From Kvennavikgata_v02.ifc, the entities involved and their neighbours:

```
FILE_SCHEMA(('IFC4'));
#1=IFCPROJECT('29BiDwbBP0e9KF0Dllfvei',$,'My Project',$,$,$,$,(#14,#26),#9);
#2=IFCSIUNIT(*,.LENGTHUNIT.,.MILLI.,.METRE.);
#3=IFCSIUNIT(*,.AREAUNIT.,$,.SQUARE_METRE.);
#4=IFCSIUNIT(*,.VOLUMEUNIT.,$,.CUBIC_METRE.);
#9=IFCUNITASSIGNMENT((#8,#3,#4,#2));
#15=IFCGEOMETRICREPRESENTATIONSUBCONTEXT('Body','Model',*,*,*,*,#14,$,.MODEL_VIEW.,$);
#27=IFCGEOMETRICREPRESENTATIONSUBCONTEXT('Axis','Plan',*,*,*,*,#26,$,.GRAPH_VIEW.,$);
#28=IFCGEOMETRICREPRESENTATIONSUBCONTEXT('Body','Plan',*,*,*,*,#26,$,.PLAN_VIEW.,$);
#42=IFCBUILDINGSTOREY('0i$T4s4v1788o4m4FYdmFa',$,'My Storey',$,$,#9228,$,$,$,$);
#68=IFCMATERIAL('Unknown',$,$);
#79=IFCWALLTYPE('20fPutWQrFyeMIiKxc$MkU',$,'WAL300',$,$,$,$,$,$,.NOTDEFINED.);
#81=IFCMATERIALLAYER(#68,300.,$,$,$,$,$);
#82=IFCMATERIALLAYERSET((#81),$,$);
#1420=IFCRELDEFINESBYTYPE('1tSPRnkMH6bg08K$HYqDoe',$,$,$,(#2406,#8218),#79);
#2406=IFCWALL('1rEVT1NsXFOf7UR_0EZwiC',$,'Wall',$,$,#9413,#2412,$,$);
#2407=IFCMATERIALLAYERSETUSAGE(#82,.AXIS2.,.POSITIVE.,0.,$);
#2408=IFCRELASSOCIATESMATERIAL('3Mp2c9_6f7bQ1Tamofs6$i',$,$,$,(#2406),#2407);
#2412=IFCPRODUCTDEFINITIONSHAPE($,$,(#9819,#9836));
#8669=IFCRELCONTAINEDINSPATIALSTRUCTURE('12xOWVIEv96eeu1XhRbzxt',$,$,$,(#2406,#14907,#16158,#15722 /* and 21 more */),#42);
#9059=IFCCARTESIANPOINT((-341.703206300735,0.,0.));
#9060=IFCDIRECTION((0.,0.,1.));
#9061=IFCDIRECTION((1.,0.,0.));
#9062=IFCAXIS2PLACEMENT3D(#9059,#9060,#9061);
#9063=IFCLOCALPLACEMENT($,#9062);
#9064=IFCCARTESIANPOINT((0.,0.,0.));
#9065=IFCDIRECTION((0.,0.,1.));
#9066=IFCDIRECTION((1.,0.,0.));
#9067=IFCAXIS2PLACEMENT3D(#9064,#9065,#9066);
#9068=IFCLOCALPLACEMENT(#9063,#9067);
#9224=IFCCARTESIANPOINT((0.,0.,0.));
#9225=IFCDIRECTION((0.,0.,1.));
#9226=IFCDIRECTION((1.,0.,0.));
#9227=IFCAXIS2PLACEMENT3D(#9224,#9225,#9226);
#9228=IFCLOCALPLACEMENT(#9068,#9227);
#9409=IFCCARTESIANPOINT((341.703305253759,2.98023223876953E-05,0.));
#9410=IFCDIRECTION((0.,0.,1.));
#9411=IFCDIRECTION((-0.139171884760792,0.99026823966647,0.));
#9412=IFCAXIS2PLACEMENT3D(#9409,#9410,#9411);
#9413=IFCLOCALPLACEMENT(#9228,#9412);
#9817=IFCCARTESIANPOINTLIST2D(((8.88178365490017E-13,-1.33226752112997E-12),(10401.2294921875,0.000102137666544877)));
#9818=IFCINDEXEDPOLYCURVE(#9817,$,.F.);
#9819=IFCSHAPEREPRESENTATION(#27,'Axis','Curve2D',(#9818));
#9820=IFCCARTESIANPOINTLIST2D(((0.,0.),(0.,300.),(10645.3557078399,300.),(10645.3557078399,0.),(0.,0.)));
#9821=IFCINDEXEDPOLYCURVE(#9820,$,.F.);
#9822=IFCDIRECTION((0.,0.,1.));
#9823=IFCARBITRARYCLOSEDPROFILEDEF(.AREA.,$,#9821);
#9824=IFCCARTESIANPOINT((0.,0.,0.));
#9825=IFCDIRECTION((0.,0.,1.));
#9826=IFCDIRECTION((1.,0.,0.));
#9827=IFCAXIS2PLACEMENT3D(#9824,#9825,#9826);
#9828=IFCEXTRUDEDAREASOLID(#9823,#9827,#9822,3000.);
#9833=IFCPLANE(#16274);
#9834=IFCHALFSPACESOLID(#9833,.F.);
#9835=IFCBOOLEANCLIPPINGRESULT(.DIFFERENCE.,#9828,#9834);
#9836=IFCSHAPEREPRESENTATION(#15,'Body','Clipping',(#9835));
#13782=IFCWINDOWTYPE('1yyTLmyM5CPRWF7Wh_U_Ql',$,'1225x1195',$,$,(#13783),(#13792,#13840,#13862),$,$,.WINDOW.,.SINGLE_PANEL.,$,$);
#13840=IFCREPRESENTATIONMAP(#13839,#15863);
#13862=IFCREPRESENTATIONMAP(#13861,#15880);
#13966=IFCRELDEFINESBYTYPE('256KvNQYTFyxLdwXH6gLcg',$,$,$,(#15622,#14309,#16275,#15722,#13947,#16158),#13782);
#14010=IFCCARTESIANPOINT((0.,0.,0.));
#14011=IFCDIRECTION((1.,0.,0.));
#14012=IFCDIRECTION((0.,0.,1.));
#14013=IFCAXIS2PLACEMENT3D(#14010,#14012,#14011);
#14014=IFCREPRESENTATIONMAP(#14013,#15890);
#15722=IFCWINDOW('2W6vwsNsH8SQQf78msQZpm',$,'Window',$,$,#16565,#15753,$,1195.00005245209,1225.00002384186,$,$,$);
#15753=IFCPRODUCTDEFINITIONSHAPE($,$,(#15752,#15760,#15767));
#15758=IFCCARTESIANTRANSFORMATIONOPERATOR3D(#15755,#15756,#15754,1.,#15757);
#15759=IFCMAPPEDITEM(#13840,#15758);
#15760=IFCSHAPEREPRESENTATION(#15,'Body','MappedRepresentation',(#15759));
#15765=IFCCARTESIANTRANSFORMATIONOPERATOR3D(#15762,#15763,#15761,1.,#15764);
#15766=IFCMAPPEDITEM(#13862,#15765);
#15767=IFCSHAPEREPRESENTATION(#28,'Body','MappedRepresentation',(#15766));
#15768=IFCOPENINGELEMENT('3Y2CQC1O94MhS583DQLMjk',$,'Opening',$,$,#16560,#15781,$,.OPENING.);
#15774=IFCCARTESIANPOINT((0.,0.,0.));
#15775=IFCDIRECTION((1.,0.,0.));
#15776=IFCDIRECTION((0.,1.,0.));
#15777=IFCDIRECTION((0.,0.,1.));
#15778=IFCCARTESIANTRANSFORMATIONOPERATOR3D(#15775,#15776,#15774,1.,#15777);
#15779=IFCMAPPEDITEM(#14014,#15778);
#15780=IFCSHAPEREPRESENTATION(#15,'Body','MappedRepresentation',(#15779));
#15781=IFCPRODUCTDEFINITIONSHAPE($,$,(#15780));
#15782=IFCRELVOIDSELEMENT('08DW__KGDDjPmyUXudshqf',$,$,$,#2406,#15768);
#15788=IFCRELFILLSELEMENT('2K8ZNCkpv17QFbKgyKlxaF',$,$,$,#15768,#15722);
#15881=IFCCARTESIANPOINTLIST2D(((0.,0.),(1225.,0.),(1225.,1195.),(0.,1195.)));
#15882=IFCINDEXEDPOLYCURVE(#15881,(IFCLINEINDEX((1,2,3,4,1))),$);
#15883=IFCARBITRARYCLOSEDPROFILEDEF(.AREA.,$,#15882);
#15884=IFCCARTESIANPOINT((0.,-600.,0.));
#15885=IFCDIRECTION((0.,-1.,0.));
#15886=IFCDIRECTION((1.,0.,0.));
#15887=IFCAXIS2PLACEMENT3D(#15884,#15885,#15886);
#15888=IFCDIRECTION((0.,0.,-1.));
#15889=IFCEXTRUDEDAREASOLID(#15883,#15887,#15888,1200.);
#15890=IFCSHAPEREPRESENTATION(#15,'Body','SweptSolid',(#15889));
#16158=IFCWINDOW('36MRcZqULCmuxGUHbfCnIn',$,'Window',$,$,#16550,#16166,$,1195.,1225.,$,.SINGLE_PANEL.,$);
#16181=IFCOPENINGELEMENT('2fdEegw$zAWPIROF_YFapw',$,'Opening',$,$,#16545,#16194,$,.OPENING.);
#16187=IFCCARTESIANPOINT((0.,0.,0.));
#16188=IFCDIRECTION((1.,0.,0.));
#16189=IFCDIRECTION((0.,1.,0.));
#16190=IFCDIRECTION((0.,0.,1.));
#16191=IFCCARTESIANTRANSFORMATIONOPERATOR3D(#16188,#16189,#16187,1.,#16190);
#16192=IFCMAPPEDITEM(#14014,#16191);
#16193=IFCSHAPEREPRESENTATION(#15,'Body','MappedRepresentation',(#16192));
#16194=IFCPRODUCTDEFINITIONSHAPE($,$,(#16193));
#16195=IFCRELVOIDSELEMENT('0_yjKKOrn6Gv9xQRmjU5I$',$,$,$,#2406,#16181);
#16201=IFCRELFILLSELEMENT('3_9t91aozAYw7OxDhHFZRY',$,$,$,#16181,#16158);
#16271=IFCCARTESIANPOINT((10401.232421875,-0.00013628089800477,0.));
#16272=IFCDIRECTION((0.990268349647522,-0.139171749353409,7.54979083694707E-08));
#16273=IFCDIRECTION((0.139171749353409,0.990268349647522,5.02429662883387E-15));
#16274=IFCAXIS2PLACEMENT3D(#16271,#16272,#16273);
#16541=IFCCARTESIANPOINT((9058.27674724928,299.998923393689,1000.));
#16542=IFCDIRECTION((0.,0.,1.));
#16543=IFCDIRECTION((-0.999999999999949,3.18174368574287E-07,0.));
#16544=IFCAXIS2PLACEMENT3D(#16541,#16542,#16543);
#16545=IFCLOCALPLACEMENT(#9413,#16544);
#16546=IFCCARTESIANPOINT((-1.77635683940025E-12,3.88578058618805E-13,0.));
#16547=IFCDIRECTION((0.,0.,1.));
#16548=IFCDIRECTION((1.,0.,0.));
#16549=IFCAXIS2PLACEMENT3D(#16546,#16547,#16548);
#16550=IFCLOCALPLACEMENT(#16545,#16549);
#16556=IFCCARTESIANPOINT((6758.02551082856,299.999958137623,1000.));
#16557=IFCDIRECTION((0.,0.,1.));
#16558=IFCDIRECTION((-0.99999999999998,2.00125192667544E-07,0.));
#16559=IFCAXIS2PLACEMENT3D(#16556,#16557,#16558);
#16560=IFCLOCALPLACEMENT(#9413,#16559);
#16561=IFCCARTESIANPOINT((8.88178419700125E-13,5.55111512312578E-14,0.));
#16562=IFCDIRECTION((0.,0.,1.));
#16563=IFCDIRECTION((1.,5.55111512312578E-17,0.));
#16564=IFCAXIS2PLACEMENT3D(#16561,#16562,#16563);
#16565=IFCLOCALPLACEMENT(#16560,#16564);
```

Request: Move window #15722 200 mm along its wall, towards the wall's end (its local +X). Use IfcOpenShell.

```python
import ifcopenshell
import ifcopenshell.api.geometry
import ifcopenshell.util.placement

model = ifcopenshell.open("Kvennavikgata_v02.ifc")

window = model.by_guid("2W6vwsNsH8SQQf78msQZpm")
opening = window.FillsVoids[0].RelatingOpeningElement
wall = opening.VoidsElements[0].RelatingBuildingElement

wall_matrix = ifcopenshell.util.placement.get_local_placement(wall.ObjectPlacement)
shift = wall_matrix[:3, 0] * 200.0
before = ifcopenshell.util.placement.get_local_placement(window.ObjectPlacement)[:3, 3].copy()

# The window is placed relative to its opening, so it follows when the opening moves.
matrix = ifcopenshell.util.placement.get_local_placement(opening.ObjectPlacement)
matrix[:3, 3] += shift
ifcopenshell.api.geometry.edit_object_placement(
    model, product=opening, matrix=matrix, is_si=False, should_transform_children=True
)

after = ifcopenshell.util.placement.get_local_placement(window.ObjectPlacement)[:3, 3]
print("window moved by", (after - before).round(3) + 0.0)

model.write("Kvennavikgata_v02_edited.ifc")
```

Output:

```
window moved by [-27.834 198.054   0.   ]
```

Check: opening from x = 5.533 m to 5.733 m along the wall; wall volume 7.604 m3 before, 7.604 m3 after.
